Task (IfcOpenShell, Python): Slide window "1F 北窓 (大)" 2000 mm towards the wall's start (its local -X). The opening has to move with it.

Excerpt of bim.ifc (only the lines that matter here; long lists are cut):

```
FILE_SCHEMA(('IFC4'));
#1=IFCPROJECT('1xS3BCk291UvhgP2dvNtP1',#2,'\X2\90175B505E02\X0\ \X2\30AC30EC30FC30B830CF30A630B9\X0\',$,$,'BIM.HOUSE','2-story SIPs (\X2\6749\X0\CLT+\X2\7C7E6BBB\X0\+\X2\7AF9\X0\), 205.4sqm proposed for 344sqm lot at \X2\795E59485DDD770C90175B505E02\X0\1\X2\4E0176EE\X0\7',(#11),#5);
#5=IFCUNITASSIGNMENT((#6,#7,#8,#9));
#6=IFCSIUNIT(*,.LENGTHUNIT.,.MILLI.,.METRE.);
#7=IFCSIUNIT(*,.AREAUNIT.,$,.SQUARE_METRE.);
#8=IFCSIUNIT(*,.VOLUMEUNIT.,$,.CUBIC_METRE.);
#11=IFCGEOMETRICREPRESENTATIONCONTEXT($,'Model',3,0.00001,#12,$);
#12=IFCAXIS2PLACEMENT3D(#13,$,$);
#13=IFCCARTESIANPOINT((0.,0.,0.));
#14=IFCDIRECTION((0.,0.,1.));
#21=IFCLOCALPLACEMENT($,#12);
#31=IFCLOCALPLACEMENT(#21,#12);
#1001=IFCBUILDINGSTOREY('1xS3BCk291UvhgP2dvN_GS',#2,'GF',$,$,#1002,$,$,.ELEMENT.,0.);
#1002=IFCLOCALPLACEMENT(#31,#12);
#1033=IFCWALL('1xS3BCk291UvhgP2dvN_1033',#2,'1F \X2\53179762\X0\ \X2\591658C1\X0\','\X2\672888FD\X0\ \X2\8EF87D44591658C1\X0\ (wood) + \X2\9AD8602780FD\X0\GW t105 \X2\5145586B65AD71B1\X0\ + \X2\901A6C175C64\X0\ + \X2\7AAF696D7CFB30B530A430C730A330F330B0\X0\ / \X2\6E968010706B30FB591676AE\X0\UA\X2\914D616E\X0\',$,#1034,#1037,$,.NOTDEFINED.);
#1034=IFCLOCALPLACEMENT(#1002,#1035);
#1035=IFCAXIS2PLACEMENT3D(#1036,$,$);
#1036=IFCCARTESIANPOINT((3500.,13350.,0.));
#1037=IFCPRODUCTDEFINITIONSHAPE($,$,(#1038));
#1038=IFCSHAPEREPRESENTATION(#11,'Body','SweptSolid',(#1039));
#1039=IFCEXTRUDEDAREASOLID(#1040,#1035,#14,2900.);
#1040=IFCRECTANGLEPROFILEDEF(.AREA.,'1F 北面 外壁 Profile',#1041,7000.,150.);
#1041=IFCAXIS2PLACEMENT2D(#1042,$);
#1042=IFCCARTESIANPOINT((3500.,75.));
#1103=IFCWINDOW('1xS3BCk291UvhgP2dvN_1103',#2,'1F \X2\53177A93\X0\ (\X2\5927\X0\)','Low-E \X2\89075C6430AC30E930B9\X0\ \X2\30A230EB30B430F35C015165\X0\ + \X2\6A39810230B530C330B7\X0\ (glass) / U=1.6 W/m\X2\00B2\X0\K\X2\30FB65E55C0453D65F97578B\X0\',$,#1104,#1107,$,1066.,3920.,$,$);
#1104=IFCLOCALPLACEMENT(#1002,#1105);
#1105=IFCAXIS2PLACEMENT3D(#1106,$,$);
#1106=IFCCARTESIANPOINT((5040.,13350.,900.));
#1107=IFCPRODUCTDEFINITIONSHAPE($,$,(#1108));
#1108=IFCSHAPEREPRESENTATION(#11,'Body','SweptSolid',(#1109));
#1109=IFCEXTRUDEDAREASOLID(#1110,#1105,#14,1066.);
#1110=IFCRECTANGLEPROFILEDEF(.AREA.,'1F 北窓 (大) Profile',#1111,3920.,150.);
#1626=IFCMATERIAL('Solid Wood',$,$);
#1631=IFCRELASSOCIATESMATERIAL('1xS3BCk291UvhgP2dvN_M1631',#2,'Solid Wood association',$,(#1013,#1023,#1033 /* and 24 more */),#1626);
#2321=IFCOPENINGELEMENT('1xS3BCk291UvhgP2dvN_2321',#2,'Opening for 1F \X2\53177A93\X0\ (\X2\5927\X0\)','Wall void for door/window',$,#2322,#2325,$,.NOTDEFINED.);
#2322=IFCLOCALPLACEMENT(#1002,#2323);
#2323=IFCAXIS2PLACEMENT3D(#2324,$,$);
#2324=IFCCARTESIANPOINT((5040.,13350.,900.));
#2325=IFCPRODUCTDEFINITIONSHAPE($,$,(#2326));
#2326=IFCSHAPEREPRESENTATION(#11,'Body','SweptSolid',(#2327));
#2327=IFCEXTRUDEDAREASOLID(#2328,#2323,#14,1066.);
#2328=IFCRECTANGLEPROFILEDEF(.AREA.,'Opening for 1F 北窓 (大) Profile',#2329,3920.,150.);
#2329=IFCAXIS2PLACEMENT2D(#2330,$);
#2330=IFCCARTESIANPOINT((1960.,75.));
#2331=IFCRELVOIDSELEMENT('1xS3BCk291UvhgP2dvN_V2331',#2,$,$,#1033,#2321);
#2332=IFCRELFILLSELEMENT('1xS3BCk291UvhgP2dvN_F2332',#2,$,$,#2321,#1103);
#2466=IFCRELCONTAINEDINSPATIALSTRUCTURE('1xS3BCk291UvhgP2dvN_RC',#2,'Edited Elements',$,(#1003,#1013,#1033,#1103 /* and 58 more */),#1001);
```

```python
import ifcopenshell
import ifcopenshell.api.geometry
import ifcopenshell.util.placement
import ifcopenshell.util.unit

model = ifcopenshell.open("bim.ifc")
unit_scale = ifcopenshell.util.unit.calculate_unit_scale(model)

window = model.by_guid("1xS3BCk291UvhgP2dvN_1103")
opening = window.FillsVoids[0].RelatingOpeningElement
wall = opening.VoidsElements[0].RelatingBuildingElement

wall_matrix = ifcopenshell.util.placement.get_local_placement(wall.ObjectPlacement)
shift = wall_matrix[:3, 0] * -2 / unit_scale
before = ifcopenshell.util.placement.get_local_placement(window.ObjectPlacement)[:3, 3].copy()

# The window is not placed relative to its opening, so move both.
for product in (opening, window):
    matrix = ifcopenshell.util.placement.get_local_placement(product.ObjectPlacement)
    matrix[:3, 3] += shift
    ifcopenshell.api.geometry.edit_object_placement(model, product=product, matrix=matrix, is_si=False)

after = ifcopenshell.util.placement.get_local_placement(window.ObjectPlacement)[:3, 3]
print("window moved by", (after - before).round(3) + 0.0)

model.write("bim_rev.ifc")
```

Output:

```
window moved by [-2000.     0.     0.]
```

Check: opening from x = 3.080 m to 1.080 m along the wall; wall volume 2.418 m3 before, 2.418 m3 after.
